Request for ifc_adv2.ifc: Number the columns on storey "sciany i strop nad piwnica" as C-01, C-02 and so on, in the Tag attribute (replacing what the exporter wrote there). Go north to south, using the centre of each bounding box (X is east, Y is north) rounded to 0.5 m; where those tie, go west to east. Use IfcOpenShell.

First a look at what the model holds.

```python
import ifcopenshell
import ifcopenshell.util.element
import ifcopenshell.util.placement

model = ifcopenshell.open("ifc_adv2.ifc")
print(model.schema)
storey = next(s for s in model.by_type("IfcBuildingStorey") if s.Name == "sciany i strop nad piwnica")
columns = [e for e in ifcopenshell.util.element.get_decomposition(storey) if e.is_a("IfcColumn")]
for e in sorted(columns, key=lambda e: e.id()):
    origin = ifcopenshell.util.placement.get_local_placement(e.ObjectPlacement)[:3, 3]
    print(e.id(), e.Tag, e.Name, origin.round(2) + 0.0, sep=" | ")
```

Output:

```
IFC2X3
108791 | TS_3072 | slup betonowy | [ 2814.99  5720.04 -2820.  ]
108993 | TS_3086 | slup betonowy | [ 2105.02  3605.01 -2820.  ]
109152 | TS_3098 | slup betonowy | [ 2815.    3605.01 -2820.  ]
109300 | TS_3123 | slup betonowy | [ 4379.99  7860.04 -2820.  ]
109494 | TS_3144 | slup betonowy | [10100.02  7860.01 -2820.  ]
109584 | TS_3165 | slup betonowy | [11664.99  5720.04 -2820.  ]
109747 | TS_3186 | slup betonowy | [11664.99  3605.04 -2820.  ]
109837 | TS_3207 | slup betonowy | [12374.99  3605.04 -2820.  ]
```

```python
import ifcopenshell
import ifcopenshell.geom
import ifcopenshell.util.element
import ifcopenshell.util.shape

model = ifcopenshell.open("ifc_adv2.ifc")
settings = ifcopenshell.geom.settings()
settings.set("use-world-coords", True)


def centre(element):
    shape = ifcopenshell.geom.create_shape(settings, element)
    return ifcopenshell.util.shape.get_bbox_centroid(shape.geometry)


storey = next(s for s in model.by_type("IfcBuildingStorey") if s.Name == "sciany i strop nad piwnica")
columns = [e for e in ifcopenshell.util.element.get_decomposition(storey) if e.is_a("IfcColumn")]

# Insertion points can sit at a corner or the storey origin, so sort by the geometry (in metres).
centres = {e: centre(e) for e in columns}
columns.sort(key=lambda e: (-round(centres[e][1] / 0.5), centres[e][0]))

for i, e in enumerate(columns, start=1):
    number = f"C-{i:02d}"
    e.Tag = number
    print(e.id(), number)

model.write("ifc_adv2_rev.ifc")
```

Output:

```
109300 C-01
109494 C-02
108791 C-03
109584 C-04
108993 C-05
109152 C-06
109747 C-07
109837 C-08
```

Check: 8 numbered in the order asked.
